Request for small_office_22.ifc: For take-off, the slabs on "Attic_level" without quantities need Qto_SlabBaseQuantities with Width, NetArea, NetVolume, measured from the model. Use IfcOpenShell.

First a look at what the model holds.

```python
import ifcopenshell
import ifcopenshell.util.element
import ifcopenshell.util.unit

model = ifcopenshell.open("small_office_22.ifc")
print(model.schema)
for unit_type in ("LENGTHUNIT", "AREAUNIT", "VOLUMEUNIT"):
    print(unit_type, ifcopenshell.util.unit.calculate_unit_scale(model, unit_type))
storey = next(s for s in model.by_type("IfcBuildingStorey") if s.Name == "Attic_level")
slabs = [e for e in ifcopenshell.util.element.get_decomposition(storey) if e.is_a("IfcSlab")]
for e in sorted(slabs, key=lambda e: e.id()):
    print(e.id(), e.is_a(), e.Name, list(ifcopenshell.util.element.get_psets(e, qtos_only=True)), sep=" | ")
```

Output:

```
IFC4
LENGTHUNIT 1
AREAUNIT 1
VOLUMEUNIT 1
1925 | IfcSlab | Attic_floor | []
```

```python
import ifcopenshell
import ifcopenshell.api.pset
import ifcopenshell.geom
import ifcopenshell.util.element
import ifcopenshell.util.shape
import ifcopenshell.util.unit

model = ifcopenshell.open("small_office_22.ifc")
unit_scale = ifcopenshell.util.unit.calculate_unit_scale(model)
area_scale = ifcopenshell.util.unit.calculate_unit_scale(model, "AREAUNIT")
volume_scale = ifcopenshell.util.unit.calculate_unit_scale(model, "VOLUMEUNIT")
settings = ifcopenshell.geom.settings()

storey = next(s for s in model.by_type("IfcBuildingStorey") if s.Name == "Attic_level")
slabs = [e for e in ifcopenshell.util.element.get_decomposition(storey) if e.is_a("IfcSlab")]

for e in sorted(slabs, key=lambda e: e.id()):
    if ifcopenshell.util.element.get_psets(e, qtos_only=True, should_inherit=False):
        continue
    # Geometry comes back in metres, in the element's own axes.
    shape = ifcopenshell.geom.create_shape(settings, e)
    values = {
        "Width": ifcopenshell.util.shape.get_z(shape.geometry) / unit_scale,
        "NetArea": ifcopenshell.util.shape.get_footprint_area(shape.geometry) / area_scale,
        "NetVolume": ifcopenshell.util.shape.get_volume(shape.geometry) / volume_scale,
    }
    qto = ifcopenshell.api.pset.add_qto(model, product=e, name="Qto_SlabBaseQuantities")
    ifcopenshell.api.pset.edit_qto(model, qto=qto, properties=values)
    print(e.id(), {k: round(v, 3) for k, v in values.items()})

model.write("small_office_22_updated.ifc")
```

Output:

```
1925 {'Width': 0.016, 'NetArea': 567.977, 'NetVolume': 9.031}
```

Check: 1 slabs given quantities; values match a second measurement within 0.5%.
